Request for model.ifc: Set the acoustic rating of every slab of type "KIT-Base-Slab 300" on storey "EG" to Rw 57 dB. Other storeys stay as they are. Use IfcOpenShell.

First a look at what the model holds.

```python
import ifcopenshell
import ifcopenshell.util.element

model = ifcopenshell.open("model.ifc")
print(model.schema)
storey = next(s for s in model.by_type("IfcBuildingStorey") if s.Name == "EG")
slabs = [e for e in ifcopenshell.util.element.get_decomposition(storey) if e.is_a("IfcSlab")]
seen = {}
for e in slabs:
    element_type = ifcopenshell.util.element.get_type(e)
    key = (element_type.Name if element_type != e and element_type else None, ifcopenshell.util.element.get_pset(e, "Pset_SlabCommon", "AcousticRating"))
    seen[key] = seen.get(key, 0) + 1
for (name, value), count in sorted(seen.items(), key=str):
    print(count, "x", name, "|", value)
```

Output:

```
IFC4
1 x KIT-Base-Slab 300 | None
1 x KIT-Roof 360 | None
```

```python
import ifcopenshell
import ifcopenshell.api.pset
import ifcopenshell.util.element

model = ifcopenshell.open("model.ifc")

storey = next(s for s in model.by_type("IfcBuildingStorey") if s.Name == "EG")
slabs = [e for e in ifcopenshell.util.element.get_decomposition(storey) if e.is_a("IfcSlab")]

count = 0
for e in slabs:
    element_type = ifcopenshell.util.element.get_type(e)
    if element_type in (None, e) or element_type.Name != "KIT-Base-Slab 300":
        continue
    # add_pset returns the element's existing set when there is one.
    pset = ifcopenshell.api.pset.add_pset(model, product=e, name="Pset_SlabCommon")
    ifcopenshell.api.pset.edit_pset(model, pset=pset, properties={"AcousticRating": "Rw 57 dB"})
    count += 1

print(count, "slabs updated")

model.write("model_updated.ifc")
```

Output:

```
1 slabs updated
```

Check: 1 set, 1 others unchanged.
